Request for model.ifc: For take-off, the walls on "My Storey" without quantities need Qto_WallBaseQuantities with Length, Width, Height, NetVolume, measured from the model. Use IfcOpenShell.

First a look at what the model holds.

```python
import ifcopenshell
import ifcopenshell.util.element
import ifcopenshell.util.unit

model = ifcopenshell.open("model.ifc")
print(model.schema)
for unit_type in ("LENGTHUNIT", "AREAUNIT", "VOLUMEUNIT"):
    print(unit_type, ifcopenshell.util.unit.calculate_unit_scale(model, unit_type))
storey = next(s for s in model.by_type("IfcBuildingStorey") if s.Name == "My Storey")
walls = [e for e in ifcopenshell.util.element.get_decomposition(storey) if e.is_a("IfcWall")]
for e in sorted(walls, key=lambda e: e.id()):
    print(e.id(), e.is_a(), e.Name, list(ifcopenshell.util.element.get_psets(e, qtos_only=True)), sep=" | ")
```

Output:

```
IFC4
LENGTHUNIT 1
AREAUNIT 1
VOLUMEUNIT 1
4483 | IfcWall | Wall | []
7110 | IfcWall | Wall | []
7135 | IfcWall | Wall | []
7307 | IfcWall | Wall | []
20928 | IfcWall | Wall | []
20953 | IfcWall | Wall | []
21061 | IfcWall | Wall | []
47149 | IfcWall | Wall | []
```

```python
import ifcopenshell
import ifcopenshell.api.pset
import ifcopenshell.geom
import ifcopenshell.util.element
import ifcopenshell.util.shape
import ifcopenshell.util.unit

model = ifcopenshell.open("model.ifc")
unit_scale = ifcopenshell.util.unit.calculate_unit_scale(model)
volume_scale = ifcopenshell.util.unit.calculate_unit_scale(model, "VOLUMEUNIT")
settings = ifcopenshell.geom.settings()

storey = next(s for s in model.by_type("IfcBuildingStorey") if s.Name == "My Storey")
walls = [e for e in ifcopenshell.util.element.get_decomposition(storey) if e.is_a("IfcWall")]

for e in sorted(walls, key=lambda e: e.id()):
    if ifcopenshell.util.element.get_psets(e, qtos_only=True, should_inherit=False):
        continue
    # Geometry comes back in metres, in the element's own axes.
    shape = ifcopenshell.geom.create_shape(settings, e)
    values = {
        "Length": ifcopenshell.util.shape.get_x(shape.geometry) / unit_scale,
        "Width": ifcopenshell.util.shape.get_y(shape.geometry) / unit_scale,
        "Height": ifcopenshell.util.shape.get_z(shape.geometry) / unit_scale,
        "NetVolume": ifcopenshell.util.shape.get_volume(shape.geometry) / volume_scale,
    }
    qto = ifcopenshell.api.pset.add_qto(model, product=e, name="Qto_WallBaseQuantities")
    ifcopenshell.api.pset.edit_qto(model, qto=qto, properties=values)
    print(e.id(), {k: round(v, 3) for k, v in values.items()})

model.write("model_rev.ifc")
```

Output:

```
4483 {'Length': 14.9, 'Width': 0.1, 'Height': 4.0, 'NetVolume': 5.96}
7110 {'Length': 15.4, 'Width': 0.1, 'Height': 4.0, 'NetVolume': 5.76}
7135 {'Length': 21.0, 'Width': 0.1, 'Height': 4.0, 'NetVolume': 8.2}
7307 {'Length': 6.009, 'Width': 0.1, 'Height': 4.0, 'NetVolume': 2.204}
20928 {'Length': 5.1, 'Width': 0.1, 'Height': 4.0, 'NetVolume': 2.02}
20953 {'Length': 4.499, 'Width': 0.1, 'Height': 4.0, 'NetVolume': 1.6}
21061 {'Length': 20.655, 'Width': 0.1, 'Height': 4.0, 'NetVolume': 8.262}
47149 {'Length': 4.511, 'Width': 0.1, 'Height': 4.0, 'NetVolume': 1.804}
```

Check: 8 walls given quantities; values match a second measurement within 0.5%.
